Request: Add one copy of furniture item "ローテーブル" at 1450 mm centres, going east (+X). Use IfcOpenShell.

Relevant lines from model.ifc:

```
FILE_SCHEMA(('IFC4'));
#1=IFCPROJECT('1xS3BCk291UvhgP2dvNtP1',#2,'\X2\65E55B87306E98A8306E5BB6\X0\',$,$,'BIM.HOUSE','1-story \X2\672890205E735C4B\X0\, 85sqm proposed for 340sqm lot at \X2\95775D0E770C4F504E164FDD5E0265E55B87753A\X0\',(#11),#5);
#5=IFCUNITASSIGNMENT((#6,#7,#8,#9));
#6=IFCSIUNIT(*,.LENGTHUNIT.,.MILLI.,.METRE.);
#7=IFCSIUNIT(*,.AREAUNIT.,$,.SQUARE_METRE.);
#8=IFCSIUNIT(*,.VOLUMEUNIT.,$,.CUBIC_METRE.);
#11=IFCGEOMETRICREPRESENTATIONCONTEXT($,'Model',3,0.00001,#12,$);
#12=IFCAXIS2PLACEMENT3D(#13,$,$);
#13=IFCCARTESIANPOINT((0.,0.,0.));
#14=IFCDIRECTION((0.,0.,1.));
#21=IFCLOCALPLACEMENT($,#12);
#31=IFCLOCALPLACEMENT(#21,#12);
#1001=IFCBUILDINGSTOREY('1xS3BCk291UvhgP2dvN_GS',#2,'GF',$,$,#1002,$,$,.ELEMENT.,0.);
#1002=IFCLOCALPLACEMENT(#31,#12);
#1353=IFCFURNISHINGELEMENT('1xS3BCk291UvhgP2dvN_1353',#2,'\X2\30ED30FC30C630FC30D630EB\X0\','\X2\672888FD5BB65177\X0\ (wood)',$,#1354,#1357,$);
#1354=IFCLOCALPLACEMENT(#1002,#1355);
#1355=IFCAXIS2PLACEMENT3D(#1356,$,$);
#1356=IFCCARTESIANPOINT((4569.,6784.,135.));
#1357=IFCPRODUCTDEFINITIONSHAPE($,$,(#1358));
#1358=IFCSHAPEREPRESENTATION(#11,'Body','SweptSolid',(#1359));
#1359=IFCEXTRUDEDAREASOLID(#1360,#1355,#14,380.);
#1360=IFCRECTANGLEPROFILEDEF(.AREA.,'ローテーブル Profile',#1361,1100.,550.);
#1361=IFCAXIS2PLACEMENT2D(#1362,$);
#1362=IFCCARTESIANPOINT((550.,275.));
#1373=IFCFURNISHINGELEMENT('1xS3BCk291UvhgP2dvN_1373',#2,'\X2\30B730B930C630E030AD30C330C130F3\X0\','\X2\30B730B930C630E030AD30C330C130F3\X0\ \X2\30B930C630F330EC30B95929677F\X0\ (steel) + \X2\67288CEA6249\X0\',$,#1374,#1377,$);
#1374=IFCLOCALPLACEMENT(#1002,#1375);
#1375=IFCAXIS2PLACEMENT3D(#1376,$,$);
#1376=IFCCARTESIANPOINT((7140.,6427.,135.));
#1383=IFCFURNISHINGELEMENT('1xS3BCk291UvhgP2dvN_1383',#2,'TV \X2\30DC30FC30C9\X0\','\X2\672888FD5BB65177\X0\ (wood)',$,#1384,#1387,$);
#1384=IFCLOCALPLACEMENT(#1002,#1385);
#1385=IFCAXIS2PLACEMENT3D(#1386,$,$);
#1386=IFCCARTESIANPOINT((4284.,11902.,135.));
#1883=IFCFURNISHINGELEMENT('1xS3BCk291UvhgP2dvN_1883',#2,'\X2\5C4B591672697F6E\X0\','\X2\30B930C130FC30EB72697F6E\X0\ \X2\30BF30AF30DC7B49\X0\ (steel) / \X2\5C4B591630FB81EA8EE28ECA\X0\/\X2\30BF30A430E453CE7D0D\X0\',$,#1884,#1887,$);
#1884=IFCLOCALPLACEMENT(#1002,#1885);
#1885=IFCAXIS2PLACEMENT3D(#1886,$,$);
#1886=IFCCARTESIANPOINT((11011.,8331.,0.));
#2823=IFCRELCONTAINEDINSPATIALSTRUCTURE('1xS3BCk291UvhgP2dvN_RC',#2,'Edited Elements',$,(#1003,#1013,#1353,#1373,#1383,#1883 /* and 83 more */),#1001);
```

```python
import numpy as np
import ifcopenshell
import ifcopenshell.api.geometry
import ifcopenshell.api.root
import ifcopenshell.util.element
import ifcopenshell.util.placement
import ifcopenshell.util.unit

model = ifcopenshell.open("model.ifc")
unit_scale = ifcopenshell.util.unit.calculate_unit_scale(model)


def reuse_history(source, copy):
    """copy_class also copies each property set's owner history, people and application; keep the originals."""
    for rel in copy.IsDefinedBy:
        if rel.is_a("IfcRelDefinesByProperties") and (history := rel.RelatingPropertyDefinition.OwnerHistory):
            rel.RelatingPropertyDefinition.OwnerHistory = source.OwnerHistory
            ifcopenshell.util.element.remove_deep2(model, history)


source = model.by_guid("1xS3BCk291UvhgP2dvN_1353")
base = ifcopenshell.util.placement.get_local_placement(source.ObjectPlacement)
step = np.array([1.0, 0.0, 0.0]) * 1.45 / unit_scale

for i in range(1, 2):
    copy = ifcopenshell.api.root.copy_class(model, product=source)
    copy.Representation = ifcopenshell.util.element.copy_deep(
        model, source.Representation, exclude=["IfcGeometricRepresentationContext", "IfcRepresentationMap"]
    )
    reuse_history(source, copy)
    matrix = base.copy()
    matrix[:3, 3] += i * step
    print("added at", matrix[:3, 3].round(3) + 0.0)
    ifcopenshell.api.geometry.edit_object_placement(model, product=copy, matrix=matrix, is_si=False)

model.write("model-out.ifc")
```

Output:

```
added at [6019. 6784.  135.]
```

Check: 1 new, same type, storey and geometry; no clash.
